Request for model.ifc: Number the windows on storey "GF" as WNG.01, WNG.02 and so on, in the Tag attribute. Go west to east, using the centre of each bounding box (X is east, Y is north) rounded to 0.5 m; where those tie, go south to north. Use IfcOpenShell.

First a look at what the model holds.

```python
import ifcopenshell
import ifcopenshell.util.element
import ifcopenshell.util.placement

model = ifcopenshell.open("model.ifc")
print(model.schema)
storey = next(s for s in model.by_type("IfcBuildingStorey") if s.Name == "GF")
windows = [e for e in ifcopenshell.util.element.get_decomposition(storey) if e.is_a("IfcWindow")]
for e in sorted(windows, key=lambda e: e.id()):
    origin = ifcopenshell.util.placement.get_local_placement(e.ObjectPlacement)[:3, 3]
    print(e.id(), e.Tag, e.Name, origin.round(2) + 0.0, sep=" | ")
```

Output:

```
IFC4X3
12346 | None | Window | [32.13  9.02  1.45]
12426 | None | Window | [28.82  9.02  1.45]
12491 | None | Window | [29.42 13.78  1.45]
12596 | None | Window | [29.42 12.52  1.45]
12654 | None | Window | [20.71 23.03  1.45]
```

```python
import ifcopenshell
import ifcopenshell.geom
import ifcopenshell.util.element
import ifcopenshell.util.shape

model = ifcopenshell.open("model.ifc")
settings = ifcopenshell.geom.settings()
settings.set("use-world-coords", True)


def centre(element):
    shape = ifcopenshell.geom.create_shape(settings, element)
    return ifcopenshell.util.shape.get_bbox_centroid(shape.geometry)


storey = next(s for s in model.by_type("IfcBuildingStorey") if s.Name == "GF")
windows = [e for e in ifcopenshell.util.element.get_decomposition(storey) if e.is_a("IfcWindow")]

# Insertion points can sit at a corner or the storey origin, so sort by the geometry (in metres).
centres = {e: centre(e) for e in windows}
windows.sort(key=lambda e: (round(centres[e][0] / 0.5), centres[e][1]))

for i, e in enumerate(windows, start=1):
    number = f"WNG.{i:02d}"
    e.Tag = number
    print(e.id(), number)

model.write("model_v2.ifc")
```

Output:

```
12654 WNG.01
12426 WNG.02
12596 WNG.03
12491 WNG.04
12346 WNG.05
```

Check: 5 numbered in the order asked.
